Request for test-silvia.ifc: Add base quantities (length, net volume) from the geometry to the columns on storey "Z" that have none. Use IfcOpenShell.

First a look at what the model holds.

```python
import ifcopenshell
import ifcopenshell.util.element
import ifcopenshell.util.unit

model = ifcopenshell.open("test-silvia.ifc")
print(model.schema)
for unit_type in ("LENGTHUNIT", "AREAUNIT", "VOLUMEUNIT"):
    print(unit_type, ifcopenshell.util.unit.calculate_unit_scale(model, unit_type))
storey = next(s for s in model.by_type("IfcBuildingStorey") if s.Name == "Z")
columns = [e for e in ifcopenshell.util.element.get_decomposition(storey) if e.is_a("IfcColumn")]
for e in sorted(columns, key=lambda e: e.id()):
    print(e.id(), e.is_a(), e.Name, list(ifcopenshell.util.element.get_psets(e, qtos_only=True)), sep=" | ")
```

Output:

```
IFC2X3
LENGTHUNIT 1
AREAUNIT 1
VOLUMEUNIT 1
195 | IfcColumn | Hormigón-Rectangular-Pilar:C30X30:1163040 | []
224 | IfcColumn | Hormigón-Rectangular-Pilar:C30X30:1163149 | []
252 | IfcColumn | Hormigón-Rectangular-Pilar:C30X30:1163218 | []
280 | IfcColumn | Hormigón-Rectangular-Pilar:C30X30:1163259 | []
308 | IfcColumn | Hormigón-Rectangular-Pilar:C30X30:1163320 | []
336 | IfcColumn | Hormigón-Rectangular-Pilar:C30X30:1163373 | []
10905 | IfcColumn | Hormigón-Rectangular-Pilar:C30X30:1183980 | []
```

```python
import ifcopenshell
import ifcopenshell.api.pset
import ifcopenshell.geom
import ifcopenshell.util.element
import ifcopenshell.util.shape
import ifcopenshell.util.unit

model = ifcopenshell.open("test-silvia.ifc")
unit_scale = ifcopenshell.util.unit.calculate_unit_scale(model)
volume_scale = ifcopenshell.util.unit.calculate_unit_scale(model, "VOLUMEUNIT")
settings = ifcopenshell.geom.settings()

storey = next(s for s in model.by_type("IfcBuildingStorey") if s.Name == "Z")
columns = [e for e in ifcopenshell.util.element.get_decomposition(storey) if e.is_a("IfcColumn")]

for e in sorted(columns, key=lambda e: e.id()):
    if ifcopenshell.util.element.get_psets(e, qtos_only=True, should_inherit=False):
        continue
    # Geometry comes back in metres, in the element's own axes.
    shape = ifcopenshell.geom.create_shape(settings, e)
    values = {
        "Length": ifcopenshell.util.shape.get_z(shape.geometry) / unit_scale,
        "NetVolume": ifcopenshell.util.shape.get_volume(shape.geometry) / volume_scale,
    }
    qto = ifcopenshell.api.pset.add_qto(model, product=e, name="BaseQuantities")
    ifcopenshell.api.pset.edit_qto(model, qto=qto, properties=values)
    print(e.id(), {k: round(v, 3) for k, v in values.items()})

model.write("test-silvia_rev.ifc")
```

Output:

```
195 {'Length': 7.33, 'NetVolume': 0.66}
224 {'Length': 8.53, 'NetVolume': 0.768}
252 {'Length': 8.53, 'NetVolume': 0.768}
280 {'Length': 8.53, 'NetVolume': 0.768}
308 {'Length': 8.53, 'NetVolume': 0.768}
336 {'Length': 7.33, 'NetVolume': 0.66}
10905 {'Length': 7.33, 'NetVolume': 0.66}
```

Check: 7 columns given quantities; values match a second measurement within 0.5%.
